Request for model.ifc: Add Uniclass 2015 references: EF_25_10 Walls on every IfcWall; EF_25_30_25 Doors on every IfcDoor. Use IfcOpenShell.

First a look at what the model holds.

```python
import ifcopenshell

model = ifcopenshell.open("model.ifc")
print(model.schema)
print("classifications:", [c.Name for c in model.by_type("IfcClassification")])
for ifc_class in ("IfcDoor", "IfcRoof", "IfcStair", "IfcWall", "IfcWindow"):
    print(ifc_class, len(model.by_type(ifc_class)))
```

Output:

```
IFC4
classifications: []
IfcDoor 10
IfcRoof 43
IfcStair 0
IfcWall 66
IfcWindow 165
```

```python
import ifcopenshell
import ifcopenshell.api.classification

model = ifcopenshell.open("model.ifc")

system = ifcopenshell.api.classification.add_classification(model, classification="Uniclass 2015")

codes = {
    "IfcWall": ("EF_25_10", "Walls"),
    "IfcDoor": ("EF_25_30_25", "Doors"),
}
for ifc_class, (code, name) in codes.items():
    products = model.by_type(ifc_class)
    ifcopenshell.api.classification.add_reference(
        model, products=products, classification=system, identification=code, name=name
    )
    print(code, len(products))

model.write("model_updated.ifc")
```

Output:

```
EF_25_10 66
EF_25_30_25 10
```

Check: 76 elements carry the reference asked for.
